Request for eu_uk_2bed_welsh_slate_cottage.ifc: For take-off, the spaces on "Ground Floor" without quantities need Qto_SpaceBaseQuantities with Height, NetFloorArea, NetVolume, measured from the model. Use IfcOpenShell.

First a look at what the model holds.

```python
import ifcopenshell
import ifcopenshell.util.element
import ifcopenshell.util.unit

model = ifcopenshell.open("eu_uk_2bed_welsh_slate_cottage.ifc")
print(model.schema)
for unit_type in ("LENGTHUNIT", "AREAUNIT", "VOLUMEUNIT"):
    print(unit_type, ifcopenshell.util.unit.calculate_unit_scale(model, unit_type))
storey = next(s for s in model.by_type("IfcBuildingStorey") if s.Name == "Ground Floor")
spaces = [e for e in ifcopenshell.util.element.get_decomposition(storey) if e.is_a("IfcSpace")]
for e in sorted(spaces, key=lambda e: e.id()):
    print(e.id(), e.is_a(), e.Name, list(ifcopenshell.util.element.get_psets(e, qtos_only=True)), sep=" | ")
```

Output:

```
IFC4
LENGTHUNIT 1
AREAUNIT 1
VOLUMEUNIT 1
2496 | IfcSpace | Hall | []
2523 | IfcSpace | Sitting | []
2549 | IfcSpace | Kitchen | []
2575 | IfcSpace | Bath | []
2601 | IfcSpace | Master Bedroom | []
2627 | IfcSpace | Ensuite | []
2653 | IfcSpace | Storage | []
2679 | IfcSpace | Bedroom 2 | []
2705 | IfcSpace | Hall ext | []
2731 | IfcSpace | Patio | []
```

```python
import ifcopenshell
import ifcopenshell.api.pset
import ifcopenshell.geom
import ifcopenshell.util.element
import ifcopenshell.util.shape
import ifcopenshell.util.unit

model = ifcopenshell.open("eu_uk_2bed_welsh_slate_cottage.ifc")
unit_scale = ifcopenshell.util.unit.calculate_unit_scale(model)
area_scale = ifcopenshell.util.unit.calculate_unit_scale(model, "AREAUNIT")
volume_scale = ifcopenshell.util.unit.calculate_unit_scale(model, "VOLUMEUNIT")
settings = ifcopenshell.geom.settings()

storey = next(s for s in model.by_type("IfcBuildingStorey") if s.Name == "Ground Floor")
spaces = [e for e in ifcopenshell.util.element.get_decomposition(storey) if e.is_a("IfcSpace")]

for e in sorted(spaces, key=lambda e: e.id()):
    if ifcopenshell.util.element.get_psets(e, qtos_only=True, should_inherit=False):
        continue
    # Geometry comes back in metres, in the element's own axes.
    shape = ifcopenshell.geom.create_shape(settings, e)
    values = {
        "Height": ifcopenshell.util.shape.get_z(shape.geometry) / unit_scale,
        "NetFloorArea": ifcopenshell.util.shape.get_footprint_area(shape.geometry) / area_scale,
        "NetVolume": ifcopenshell.util.shape.get_volume(shape.geometry) / volume_scale,
    }
    qto = ifcopenshell.api.pset.add_qto(model, product=e, name="Qto_SpaceBaseQuantities")
    ifcopenshell.api.pset.edit_qto(model, qto=qto, properties=values)
    print(e.id(), {k: round(v, 3) for k, v in values.items()})

model.write("eu_uk_2bed_welsh_slate_cottage_edited.ifc")
```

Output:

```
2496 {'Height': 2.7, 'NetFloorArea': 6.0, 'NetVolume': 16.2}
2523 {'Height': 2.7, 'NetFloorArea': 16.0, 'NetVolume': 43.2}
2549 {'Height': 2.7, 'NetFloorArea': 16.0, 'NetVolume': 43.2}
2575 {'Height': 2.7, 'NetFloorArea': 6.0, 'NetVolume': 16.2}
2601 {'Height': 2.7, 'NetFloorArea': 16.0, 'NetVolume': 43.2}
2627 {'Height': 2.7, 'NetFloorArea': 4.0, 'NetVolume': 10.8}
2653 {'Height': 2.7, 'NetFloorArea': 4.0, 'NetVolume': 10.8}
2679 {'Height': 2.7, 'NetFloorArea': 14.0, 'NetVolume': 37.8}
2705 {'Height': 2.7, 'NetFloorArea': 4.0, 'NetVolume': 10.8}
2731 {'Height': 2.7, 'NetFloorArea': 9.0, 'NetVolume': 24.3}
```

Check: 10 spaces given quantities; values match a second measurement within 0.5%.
